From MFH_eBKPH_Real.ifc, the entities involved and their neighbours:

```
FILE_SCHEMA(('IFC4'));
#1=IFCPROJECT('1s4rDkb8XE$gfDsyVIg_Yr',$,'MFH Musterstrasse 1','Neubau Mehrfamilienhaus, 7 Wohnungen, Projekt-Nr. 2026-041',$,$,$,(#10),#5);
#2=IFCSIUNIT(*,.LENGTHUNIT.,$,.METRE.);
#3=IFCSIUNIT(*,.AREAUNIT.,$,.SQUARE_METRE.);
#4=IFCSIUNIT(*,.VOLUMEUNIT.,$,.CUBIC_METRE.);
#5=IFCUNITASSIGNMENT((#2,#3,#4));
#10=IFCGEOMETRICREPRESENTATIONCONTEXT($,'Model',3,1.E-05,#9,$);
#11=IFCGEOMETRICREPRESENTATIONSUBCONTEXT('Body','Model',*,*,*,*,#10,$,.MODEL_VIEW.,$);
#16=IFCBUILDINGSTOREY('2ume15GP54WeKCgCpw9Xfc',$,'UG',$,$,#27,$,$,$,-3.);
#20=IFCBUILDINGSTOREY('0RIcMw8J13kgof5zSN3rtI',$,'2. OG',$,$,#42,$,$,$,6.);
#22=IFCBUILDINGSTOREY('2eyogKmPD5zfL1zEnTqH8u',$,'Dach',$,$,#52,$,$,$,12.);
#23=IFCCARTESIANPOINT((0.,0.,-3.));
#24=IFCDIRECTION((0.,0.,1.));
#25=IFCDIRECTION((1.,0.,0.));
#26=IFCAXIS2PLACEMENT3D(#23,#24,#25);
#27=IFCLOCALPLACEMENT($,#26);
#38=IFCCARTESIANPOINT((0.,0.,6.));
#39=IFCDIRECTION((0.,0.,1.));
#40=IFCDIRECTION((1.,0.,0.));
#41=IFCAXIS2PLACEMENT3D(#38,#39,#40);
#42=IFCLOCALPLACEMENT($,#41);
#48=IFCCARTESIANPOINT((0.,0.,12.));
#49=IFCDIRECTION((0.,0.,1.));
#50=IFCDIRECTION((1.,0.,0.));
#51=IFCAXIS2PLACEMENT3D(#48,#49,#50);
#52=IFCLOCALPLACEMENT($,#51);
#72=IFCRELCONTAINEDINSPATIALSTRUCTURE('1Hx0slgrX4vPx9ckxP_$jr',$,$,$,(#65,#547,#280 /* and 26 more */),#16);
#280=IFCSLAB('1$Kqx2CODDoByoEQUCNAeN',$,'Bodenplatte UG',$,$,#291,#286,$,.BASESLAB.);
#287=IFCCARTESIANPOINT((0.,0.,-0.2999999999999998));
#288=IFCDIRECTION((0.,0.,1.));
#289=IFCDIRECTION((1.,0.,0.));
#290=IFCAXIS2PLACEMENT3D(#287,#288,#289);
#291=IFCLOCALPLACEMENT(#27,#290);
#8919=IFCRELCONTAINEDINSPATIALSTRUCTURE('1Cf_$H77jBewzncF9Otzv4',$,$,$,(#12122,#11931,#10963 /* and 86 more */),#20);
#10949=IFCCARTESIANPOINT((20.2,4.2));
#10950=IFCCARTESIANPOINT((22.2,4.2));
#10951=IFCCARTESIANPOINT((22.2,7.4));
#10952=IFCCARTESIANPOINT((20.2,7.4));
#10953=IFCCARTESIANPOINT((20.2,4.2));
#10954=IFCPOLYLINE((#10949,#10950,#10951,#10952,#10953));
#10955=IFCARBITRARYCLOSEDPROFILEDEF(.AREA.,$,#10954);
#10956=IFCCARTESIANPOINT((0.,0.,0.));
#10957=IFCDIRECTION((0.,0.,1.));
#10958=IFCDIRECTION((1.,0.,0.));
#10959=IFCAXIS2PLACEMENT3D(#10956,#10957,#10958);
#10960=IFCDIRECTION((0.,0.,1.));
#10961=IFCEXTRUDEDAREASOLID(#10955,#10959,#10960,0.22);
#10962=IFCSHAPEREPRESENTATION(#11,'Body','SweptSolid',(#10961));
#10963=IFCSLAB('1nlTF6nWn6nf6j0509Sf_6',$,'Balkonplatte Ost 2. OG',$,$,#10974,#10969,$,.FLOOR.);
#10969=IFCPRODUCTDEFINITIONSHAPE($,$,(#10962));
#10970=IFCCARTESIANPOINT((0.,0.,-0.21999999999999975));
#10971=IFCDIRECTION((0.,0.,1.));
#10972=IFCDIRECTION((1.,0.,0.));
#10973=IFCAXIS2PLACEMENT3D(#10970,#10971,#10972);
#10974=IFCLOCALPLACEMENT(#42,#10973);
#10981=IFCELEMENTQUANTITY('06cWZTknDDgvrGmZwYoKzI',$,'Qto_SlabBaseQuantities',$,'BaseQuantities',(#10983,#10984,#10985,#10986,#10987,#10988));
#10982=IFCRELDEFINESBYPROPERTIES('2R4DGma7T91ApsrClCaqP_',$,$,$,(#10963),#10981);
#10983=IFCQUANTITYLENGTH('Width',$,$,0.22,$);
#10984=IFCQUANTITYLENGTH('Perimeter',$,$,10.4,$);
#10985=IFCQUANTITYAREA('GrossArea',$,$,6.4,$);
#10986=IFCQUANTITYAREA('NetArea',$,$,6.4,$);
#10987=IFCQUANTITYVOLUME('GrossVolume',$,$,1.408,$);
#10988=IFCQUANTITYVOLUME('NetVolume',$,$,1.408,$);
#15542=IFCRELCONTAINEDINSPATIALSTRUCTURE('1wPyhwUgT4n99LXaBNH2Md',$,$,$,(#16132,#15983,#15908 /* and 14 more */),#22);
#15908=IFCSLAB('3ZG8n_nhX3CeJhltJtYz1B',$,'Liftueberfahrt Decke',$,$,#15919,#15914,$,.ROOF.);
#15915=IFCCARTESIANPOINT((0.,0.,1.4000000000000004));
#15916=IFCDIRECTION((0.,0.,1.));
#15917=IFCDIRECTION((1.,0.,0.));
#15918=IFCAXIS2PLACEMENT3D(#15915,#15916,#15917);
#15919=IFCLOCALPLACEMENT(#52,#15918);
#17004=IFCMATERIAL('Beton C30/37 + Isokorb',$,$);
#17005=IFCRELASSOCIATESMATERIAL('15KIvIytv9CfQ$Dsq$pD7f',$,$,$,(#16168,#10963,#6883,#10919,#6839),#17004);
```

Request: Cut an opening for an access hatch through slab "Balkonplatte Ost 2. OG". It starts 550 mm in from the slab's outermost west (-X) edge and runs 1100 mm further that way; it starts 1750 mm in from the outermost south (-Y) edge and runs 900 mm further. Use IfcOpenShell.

```python
import numpy as np
import ifcopenshell
import ifcopenshell.api.feature
import ifcopenshell.api.geometry
import ifcopenshell.api.pset
import ifcopenshell.api.root
import ifcopenshell.geom
import ifcopenshell.util.element
import ifcopenshell.util.placement
import ifcopenshell.util.representation
import ifcopenshell.util.shape
import ifcopenshell.util.unit

model = ifcopenshell.open("MFH_eBKPH_Real.ifc")
unit_scale = ifcopenshell.util.unit.calculate_unit_scale(model)
area_scale = ifcopenshell.util.unit.calculate_unit_scale(model, "AREAUNIT")
volume_scale = ifcopenshell.util.unit.calculate_unit_scale(model, "VOLUMEUNIT")
settings = ifcopenshell.geom.settings()


def volume(element):
    """Net volume in cubic metres, openings subtracted."""
    shape = ifcopenshell.geom.create_shape(settings, element)
    return ifcopenshell.util.shape.get_volume(shape.geometry)


slab = model.by_guid("1nlTF6nWn6nf6j0509Sf_6")
before = volume(slab)

# Extent in the slab's own axes, in metres. The edges named are its -X and -Y sides.
slab_shape = ifcopenshell.geom.create_shape(settings, slab)
vertices = ifcopenshell.util.shape.get_vertices(slab_shape.geometry)
x_min, y_min, bottom = vertices.min(axis=0)
top = vertices[:, 2].max()

opening = ifcopenshell.api.root.create_entity(model, ifc_class="IfcOpeningElement", name="Access hatch opening", predefined_type="OPENING")
context = ifcopenshell.util.representation.get_context(model, "Model", "Body", "MODEL_VIEW")
width, depth = 1.1, 0.9
outline = [(0.0, 0.0), (width, 0.0), (width, depth), (0.0, depth), (0.0, 0.0)]
# Overshoot both faces by 50 mm so the cut is clean.
shape = ifcopenshell.api.geometry.add_slab_representation(
    model, context=context, depth=top - bottom + 0.1, polyline=outline
)
ifcopenshell.api.geometry.assign_representation(model, product=opening, representation=shape)

matrix = ifcopenshell.util.placement.get_local_placement(slab.ObjectPlacement)
matrix[:, 3] = matrix @ np.append(np.array([x_min + 0.55, y_min + 1.75, bottom - 0.05]) / unit_scale, 1.0)
ifcopenshell.api.geometry.edit_object_placement(model, product=opening, matrix=matrix, is_si=False)
ifcopenshell.api.feature.add_feature(model, feature=opening, element=slab)

after = volume(slab)

# Update the slab's stored quantities.
qto = model.by_id(ifcopenshell.util.element.get_pset(slab, "Qto_SlabBaseQuantities", should_inherit=False)["id"])
ifcopenshell.api.pset.edit_qto(model, qto=qto, properties={
    "NetArea": after / (top - bottom) / area_scale,
    "NetVolume": after / volume_scale,
})

print(f"slab volume {before:.3f} -> {after:.3f} m3")

model.write("MFH_eBKPH_Real-out.ifc")
```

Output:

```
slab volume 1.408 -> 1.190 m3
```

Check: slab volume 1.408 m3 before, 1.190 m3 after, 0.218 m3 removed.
